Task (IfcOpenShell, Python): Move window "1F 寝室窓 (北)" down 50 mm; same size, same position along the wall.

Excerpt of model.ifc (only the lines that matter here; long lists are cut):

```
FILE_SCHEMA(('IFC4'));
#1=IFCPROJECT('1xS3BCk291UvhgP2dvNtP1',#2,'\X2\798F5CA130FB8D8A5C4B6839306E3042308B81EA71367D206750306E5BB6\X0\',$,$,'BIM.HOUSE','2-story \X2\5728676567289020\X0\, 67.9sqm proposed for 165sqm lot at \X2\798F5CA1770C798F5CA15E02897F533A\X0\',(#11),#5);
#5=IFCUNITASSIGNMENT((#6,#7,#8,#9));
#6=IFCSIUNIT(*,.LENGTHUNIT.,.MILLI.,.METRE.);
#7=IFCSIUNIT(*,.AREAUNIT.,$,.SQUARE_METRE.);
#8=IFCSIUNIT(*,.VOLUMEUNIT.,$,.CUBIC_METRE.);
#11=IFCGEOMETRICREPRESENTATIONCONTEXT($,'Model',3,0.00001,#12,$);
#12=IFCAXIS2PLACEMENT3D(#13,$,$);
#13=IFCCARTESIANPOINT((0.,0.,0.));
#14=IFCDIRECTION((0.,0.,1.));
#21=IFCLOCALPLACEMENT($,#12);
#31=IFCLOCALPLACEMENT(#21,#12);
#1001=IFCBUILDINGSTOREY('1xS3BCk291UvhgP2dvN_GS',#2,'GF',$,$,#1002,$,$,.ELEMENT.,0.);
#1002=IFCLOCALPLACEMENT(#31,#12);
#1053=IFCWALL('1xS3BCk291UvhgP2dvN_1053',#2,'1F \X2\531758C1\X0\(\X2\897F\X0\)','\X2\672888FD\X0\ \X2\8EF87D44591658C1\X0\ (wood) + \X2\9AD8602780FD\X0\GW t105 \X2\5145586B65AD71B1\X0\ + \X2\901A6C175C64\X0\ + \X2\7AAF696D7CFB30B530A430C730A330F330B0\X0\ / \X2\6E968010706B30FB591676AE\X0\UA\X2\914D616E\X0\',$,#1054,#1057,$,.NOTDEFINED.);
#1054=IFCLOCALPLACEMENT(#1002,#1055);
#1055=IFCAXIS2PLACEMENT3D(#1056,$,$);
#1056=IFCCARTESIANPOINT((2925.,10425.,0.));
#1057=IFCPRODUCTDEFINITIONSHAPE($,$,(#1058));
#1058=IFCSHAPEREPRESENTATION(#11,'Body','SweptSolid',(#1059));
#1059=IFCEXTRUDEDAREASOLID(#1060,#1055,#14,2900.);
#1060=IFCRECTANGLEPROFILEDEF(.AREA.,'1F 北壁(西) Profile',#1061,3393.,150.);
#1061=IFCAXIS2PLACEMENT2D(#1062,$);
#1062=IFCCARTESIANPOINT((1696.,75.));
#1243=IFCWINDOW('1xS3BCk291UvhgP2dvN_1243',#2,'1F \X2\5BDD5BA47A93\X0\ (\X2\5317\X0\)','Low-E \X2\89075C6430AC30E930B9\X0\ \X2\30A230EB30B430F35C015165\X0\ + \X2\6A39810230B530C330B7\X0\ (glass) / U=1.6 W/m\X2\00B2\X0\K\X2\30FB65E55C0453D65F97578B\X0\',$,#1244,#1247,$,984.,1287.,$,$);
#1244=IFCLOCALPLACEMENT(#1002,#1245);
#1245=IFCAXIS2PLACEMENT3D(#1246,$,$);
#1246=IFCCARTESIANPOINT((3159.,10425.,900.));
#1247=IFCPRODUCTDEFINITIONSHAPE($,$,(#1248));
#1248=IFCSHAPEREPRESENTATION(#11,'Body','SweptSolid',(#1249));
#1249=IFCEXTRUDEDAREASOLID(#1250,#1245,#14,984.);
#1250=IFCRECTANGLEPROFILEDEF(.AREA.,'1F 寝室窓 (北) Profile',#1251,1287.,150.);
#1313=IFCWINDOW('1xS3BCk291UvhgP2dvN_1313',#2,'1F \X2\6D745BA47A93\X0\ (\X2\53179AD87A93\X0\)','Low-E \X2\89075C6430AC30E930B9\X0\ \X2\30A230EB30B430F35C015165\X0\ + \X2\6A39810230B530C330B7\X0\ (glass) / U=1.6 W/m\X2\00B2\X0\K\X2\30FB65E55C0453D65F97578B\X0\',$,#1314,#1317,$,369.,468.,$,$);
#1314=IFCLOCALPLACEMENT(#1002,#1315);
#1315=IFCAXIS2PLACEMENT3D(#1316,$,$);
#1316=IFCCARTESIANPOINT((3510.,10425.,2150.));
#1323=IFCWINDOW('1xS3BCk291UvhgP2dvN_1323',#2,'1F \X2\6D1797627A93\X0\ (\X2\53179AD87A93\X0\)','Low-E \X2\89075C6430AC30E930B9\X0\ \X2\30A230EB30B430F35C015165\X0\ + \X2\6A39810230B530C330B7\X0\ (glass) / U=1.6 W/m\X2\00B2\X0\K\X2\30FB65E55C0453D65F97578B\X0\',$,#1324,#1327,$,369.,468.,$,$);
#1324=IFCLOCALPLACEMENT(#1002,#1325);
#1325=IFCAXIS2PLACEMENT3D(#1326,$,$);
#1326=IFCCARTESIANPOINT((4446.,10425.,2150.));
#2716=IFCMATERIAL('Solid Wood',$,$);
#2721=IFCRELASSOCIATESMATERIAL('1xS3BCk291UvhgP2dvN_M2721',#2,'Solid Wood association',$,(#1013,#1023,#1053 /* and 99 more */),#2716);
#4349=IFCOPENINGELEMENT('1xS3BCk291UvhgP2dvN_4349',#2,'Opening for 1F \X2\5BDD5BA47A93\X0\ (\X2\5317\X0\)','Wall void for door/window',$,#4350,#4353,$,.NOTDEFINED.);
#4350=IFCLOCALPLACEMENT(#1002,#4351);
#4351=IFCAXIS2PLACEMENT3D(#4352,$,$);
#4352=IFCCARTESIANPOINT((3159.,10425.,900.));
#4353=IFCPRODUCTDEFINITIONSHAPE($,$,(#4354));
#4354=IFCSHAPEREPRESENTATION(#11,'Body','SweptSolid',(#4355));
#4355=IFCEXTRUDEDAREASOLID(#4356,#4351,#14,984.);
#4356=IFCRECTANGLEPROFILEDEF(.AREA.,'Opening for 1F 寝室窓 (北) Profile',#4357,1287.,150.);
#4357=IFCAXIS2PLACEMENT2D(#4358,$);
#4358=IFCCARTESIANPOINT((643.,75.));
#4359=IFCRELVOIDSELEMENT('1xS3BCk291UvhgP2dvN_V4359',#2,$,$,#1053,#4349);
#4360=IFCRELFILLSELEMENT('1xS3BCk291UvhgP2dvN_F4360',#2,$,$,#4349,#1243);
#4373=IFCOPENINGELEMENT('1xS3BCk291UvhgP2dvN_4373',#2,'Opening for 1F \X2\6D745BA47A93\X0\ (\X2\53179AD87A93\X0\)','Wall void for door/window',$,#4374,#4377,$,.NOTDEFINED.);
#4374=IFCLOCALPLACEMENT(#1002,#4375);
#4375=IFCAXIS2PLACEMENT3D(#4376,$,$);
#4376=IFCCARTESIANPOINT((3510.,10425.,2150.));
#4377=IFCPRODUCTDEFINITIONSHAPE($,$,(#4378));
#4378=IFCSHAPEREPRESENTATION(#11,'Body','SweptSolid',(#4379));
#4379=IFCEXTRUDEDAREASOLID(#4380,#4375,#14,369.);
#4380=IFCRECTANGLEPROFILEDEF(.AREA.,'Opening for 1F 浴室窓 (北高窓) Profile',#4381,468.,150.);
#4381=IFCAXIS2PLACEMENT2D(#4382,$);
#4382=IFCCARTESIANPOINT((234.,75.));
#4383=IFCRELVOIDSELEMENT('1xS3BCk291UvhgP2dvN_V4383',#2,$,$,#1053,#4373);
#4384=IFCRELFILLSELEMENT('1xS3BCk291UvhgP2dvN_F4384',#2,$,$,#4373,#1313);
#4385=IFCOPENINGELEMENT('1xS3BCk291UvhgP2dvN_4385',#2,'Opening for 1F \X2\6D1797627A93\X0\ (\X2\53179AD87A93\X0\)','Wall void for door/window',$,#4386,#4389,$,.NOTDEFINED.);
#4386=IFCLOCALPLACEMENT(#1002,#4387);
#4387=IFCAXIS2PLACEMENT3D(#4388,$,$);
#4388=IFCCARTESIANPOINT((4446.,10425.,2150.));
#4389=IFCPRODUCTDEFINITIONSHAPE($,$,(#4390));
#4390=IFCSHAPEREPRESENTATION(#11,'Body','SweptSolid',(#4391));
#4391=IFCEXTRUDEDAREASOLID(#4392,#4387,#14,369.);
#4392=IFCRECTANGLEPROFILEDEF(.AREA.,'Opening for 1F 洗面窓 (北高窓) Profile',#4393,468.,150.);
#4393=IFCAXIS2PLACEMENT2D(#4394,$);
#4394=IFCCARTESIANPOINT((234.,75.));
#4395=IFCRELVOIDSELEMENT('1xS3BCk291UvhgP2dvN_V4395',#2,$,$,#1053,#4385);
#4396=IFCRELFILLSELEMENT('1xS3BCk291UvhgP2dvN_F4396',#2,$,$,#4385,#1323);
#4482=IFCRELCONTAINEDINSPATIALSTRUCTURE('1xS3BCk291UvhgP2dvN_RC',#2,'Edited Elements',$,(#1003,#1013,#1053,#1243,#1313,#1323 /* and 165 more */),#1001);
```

```python
import numpy as np
import ifcopenshell
import ifcopenshell.api.geometry
import ifcopenshell.util.placement
import ifcopenshell.util.unit

model = ifcopenshell.open("model.ifc")
unit_scale = ifcopenshell.util.unit.calculate_unit_scale(model)

window = model.by_id(1243)
opening = window.FillsVoids[0].RelatingOpeningElement
dz = -50.0

shift = np.array([0.0, 0.0, dz])
# The window is not placed relative to its opening, so move both.
for product in (opening, window):
    matrix = ifcopenshell.util.placement.get_local_placement(product.ObjectPlacement)
    matrix[:3, 3] += shift
    ifcopenshell.api.geometry.edit_object_placement(model, product=product, matrix=matrix, is_si=False)

print(f"moved by {dz * unit_scale:+.3f} m")

model.write("model_updated.ifc")
```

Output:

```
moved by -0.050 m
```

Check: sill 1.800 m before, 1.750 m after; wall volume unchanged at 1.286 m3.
